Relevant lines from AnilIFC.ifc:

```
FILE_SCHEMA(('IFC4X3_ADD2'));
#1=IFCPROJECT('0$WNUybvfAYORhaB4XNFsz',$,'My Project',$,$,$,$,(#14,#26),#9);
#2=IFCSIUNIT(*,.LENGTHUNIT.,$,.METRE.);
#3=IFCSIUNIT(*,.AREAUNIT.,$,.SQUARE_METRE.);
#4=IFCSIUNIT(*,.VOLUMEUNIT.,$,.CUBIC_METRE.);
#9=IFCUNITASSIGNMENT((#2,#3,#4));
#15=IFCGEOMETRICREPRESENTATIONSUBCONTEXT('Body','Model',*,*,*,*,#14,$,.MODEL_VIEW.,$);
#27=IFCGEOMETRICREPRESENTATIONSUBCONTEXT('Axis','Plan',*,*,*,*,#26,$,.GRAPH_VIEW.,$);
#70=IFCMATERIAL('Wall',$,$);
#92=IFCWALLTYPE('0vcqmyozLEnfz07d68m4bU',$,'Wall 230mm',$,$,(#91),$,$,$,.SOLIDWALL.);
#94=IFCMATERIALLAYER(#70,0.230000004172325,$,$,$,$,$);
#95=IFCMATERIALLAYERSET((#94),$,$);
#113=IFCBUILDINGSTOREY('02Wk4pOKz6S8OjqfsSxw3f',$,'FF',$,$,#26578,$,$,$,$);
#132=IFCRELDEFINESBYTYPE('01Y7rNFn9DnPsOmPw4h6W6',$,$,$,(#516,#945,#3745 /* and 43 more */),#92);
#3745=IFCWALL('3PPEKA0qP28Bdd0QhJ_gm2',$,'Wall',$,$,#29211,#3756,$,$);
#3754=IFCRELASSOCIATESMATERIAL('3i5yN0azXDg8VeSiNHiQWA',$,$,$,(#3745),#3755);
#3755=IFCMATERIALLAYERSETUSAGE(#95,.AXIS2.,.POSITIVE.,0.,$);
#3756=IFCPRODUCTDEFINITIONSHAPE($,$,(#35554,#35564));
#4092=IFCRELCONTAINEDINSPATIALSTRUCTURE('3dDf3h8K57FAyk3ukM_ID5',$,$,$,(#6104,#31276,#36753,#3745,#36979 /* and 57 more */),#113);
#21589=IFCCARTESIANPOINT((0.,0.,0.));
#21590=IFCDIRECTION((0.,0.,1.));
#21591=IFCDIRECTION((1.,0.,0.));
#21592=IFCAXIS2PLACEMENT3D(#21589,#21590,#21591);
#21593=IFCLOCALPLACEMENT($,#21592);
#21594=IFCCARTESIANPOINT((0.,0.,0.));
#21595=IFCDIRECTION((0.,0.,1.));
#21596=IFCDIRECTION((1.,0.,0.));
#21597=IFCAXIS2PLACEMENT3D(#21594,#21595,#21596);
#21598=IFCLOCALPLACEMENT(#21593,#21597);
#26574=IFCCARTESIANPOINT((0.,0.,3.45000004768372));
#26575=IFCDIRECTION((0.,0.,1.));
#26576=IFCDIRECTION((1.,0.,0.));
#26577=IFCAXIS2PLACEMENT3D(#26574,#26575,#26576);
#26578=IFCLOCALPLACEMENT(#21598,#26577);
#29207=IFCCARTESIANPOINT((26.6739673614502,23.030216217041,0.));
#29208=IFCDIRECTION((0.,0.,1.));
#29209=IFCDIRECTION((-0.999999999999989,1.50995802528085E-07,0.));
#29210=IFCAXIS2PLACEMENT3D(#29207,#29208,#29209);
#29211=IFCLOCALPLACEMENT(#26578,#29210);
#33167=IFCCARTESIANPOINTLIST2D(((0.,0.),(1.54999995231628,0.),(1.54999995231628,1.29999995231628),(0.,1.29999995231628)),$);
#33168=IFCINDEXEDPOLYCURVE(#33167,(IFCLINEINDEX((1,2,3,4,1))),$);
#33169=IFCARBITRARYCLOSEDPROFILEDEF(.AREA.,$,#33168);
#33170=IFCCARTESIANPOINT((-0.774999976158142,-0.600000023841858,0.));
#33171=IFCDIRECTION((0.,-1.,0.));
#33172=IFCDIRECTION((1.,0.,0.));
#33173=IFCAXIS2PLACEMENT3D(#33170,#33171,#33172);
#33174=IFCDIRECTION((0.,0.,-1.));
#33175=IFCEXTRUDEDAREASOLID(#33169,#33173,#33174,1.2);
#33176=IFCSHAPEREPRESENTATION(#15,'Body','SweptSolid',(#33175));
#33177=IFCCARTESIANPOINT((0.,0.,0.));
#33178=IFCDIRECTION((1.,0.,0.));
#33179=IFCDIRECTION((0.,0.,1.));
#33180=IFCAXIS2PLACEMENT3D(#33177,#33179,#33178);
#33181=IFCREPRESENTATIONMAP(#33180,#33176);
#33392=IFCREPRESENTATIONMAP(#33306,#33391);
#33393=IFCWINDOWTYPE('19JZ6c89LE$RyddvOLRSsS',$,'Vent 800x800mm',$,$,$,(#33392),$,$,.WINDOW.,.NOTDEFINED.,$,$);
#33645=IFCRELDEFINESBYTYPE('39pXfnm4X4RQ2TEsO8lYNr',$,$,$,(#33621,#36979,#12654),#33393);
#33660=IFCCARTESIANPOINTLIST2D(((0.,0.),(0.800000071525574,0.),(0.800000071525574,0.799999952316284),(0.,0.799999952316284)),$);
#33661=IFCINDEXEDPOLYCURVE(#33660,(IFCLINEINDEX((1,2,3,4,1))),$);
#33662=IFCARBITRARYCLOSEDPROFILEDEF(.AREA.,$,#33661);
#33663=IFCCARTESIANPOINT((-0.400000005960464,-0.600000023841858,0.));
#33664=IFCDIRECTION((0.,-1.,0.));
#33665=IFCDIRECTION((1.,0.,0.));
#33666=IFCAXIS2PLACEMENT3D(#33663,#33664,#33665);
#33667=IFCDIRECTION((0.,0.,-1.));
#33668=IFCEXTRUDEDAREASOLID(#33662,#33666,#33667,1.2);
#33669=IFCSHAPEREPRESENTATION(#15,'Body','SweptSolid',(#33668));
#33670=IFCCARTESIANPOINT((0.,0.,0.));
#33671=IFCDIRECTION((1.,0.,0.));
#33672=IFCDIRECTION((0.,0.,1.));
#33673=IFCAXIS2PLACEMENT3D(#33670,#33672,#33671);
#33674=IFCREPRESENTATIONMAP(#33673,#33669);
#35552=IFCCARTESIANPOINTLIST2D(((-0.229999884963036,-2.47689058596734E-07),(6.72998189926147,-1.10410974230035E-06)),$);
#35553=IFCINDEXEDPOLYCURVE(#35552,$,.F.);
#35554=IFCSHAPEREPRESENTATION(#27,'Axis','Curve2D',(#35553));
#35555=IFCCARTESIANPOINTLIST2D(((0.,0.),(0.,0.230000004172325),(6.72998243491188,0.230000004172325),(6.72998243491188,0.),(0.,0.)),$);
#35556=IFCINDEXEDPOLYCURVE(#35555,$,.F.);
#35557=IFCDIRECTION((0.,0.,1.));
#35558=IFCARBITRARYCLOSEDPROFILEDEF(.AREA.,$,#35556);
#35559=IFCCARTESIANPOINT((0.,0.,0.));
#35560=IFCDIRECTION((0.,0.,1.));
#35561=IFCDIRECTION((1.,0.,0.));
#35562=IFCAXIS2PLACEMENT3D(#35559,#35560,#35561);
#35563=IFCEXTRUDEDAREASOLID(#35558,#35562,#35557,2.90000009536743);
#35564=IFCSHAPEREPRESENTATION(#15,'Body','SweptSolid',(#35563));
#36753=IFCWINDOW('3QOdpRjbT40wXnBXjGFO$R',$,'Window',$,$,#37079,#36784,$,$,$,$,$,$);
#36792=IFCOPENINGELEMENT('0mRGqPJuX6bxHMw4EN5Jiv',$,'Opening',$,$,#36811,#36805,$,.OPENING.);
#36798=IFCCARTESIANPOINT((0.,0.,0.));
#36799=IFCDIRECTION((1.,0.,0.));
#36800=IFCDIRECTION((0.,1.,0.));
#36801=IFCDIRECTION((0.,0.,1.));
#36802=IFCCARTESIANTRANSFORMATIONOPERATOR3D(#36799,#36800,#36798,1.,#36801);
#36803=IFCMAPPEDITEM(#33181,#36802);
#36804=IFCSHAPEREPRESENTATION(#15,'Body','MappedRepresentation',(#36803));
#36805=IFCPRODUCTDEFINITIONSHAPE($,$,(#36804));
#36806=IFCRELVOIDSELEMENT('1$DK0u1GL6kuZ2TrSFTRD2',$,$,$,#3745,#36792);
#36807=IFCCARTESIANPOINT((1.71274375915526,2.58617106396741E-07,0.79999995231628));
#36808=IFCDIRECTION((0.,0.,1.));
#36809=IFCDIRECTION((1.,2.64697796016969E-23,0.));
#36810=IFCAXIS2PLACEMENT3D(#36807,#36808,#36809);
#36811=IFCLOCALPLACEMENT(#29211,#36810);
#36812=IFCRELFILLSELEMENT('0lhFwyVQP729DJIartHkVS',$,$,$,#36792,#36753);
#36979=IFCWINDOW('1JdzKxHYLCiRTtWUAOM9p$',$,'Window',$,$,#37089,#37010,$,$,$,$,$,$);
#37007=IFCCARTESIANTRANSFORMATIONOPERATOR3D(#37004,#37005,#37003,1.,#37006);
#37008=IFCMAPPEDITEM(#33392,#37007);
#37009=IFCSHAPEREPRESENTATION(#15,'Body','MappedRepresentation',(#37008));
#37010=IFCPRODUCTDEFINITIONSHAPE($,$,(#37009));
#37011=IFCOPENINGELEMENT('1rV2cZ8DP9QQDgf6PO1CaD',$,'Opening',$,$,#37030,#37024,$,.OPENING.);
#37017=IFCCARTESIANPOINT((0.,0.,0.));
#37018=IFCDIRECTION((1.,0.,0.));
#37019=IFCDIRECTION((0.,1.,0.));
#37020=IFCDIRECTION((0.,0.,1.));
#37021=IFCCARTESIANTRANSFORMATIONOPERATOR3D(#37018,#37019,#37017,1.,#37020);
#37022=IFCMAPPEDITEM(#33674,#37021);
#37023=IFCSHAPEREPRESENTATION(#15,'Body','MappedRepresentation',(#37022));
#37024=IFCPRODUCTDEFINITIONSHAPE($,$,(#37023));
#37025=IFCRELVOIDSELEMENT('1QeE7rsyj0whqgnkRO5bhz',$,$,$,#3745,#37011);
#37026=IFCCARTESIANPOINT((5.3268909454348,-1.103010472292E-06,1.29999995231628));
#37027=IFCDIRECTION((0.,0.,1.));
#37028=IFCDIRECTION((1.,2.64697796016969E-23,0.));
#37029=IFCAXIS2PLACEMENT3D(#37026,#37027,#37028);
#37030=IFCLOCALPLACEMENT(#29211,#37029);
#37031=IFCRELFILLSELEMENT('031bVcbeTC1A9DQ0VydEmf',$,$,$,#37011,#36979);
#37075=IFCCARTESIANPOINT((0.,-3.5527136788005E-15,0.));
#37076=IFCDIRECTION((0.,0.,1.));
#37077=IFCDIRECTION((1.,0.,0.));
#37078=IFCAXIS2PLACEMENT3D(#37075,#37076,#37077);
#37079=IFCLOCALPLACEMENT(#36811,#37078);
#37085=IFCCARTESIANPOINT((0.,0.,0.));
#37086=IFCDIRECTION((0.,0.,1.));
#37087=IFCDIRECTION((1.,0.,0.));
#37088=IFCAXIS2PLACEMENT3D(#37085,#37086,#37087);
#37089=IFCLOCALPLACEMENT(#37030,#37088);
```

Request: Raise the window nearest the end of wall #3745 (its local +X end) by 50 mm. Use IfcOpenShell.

```python
import numpy as np
import ifcopenshell
import ifcopenshell.api.geometry
import ifcopenshell.util.placement
import ifcopenshell.util.unit

model = ifcopenshell.open("AnilIFC.ifc")
unit_scale = ifcopenshell.util.unit.calculate_unit_scale(model)

window = model.by_guid("1JdzKxHYLCiRTtWUAOM9p$")
opening = window.FillsVoids[0].RelatingOpeningElement
dz = 0.05 / unit_scale

shift = np.array([0.0, 0.0, dz])
# The window is placed relative to its opening, so it follows when the opening moves.
matrix = ifcopenshell.util.placement.get_local_placement(opening.ObjectPlacement)
matrix[:3, 3] += shift
ifcopenshell.api.geometry.edit_object_placement(
    model, product=opening, matrix=matrix, is_si=False, should_transform_children=True
)

print(f"moved by {dz * unit_scale:+.3f} m")

model.write("AnilIFC_updated.ifc")
```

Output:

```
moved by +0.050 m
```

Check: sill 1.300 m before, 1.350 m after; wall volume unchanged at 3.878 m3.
